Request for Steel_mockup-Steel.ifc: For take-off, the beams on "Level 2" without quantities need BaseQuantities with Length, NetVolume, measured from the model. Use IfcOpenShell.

First a look at what the model holds.

```python
import ifcopenshell
import ifcopenshell.util.element
import ifcopenshell.util.unit

model = ifcopenshell.open("Steel_mockup-Steel.ifc")
print(model.schema)
for unit_type in ("LENGTHUNIT", "AREAUNIT", "VOLUMEUNIT"):
    print(unit_type, ifcopenshell.util.unit.calculate_unit_scale(model, unit_type))
storey = next(s for s in model.by_type("IfcBuildingStorey") if s.Name == "Level 2")
beams = [e for e in ifcopenshell.util.element.get_decomposition(storey) if e.is_a("IfcBeam")]
for e in sorted(beams, key=lambda e: e.id()):
    print(e.id(), e.is_a(), e.Name, list(ifcopenshell.util.element.get_psets(e, qtos_only=True)), sep=" | ")
```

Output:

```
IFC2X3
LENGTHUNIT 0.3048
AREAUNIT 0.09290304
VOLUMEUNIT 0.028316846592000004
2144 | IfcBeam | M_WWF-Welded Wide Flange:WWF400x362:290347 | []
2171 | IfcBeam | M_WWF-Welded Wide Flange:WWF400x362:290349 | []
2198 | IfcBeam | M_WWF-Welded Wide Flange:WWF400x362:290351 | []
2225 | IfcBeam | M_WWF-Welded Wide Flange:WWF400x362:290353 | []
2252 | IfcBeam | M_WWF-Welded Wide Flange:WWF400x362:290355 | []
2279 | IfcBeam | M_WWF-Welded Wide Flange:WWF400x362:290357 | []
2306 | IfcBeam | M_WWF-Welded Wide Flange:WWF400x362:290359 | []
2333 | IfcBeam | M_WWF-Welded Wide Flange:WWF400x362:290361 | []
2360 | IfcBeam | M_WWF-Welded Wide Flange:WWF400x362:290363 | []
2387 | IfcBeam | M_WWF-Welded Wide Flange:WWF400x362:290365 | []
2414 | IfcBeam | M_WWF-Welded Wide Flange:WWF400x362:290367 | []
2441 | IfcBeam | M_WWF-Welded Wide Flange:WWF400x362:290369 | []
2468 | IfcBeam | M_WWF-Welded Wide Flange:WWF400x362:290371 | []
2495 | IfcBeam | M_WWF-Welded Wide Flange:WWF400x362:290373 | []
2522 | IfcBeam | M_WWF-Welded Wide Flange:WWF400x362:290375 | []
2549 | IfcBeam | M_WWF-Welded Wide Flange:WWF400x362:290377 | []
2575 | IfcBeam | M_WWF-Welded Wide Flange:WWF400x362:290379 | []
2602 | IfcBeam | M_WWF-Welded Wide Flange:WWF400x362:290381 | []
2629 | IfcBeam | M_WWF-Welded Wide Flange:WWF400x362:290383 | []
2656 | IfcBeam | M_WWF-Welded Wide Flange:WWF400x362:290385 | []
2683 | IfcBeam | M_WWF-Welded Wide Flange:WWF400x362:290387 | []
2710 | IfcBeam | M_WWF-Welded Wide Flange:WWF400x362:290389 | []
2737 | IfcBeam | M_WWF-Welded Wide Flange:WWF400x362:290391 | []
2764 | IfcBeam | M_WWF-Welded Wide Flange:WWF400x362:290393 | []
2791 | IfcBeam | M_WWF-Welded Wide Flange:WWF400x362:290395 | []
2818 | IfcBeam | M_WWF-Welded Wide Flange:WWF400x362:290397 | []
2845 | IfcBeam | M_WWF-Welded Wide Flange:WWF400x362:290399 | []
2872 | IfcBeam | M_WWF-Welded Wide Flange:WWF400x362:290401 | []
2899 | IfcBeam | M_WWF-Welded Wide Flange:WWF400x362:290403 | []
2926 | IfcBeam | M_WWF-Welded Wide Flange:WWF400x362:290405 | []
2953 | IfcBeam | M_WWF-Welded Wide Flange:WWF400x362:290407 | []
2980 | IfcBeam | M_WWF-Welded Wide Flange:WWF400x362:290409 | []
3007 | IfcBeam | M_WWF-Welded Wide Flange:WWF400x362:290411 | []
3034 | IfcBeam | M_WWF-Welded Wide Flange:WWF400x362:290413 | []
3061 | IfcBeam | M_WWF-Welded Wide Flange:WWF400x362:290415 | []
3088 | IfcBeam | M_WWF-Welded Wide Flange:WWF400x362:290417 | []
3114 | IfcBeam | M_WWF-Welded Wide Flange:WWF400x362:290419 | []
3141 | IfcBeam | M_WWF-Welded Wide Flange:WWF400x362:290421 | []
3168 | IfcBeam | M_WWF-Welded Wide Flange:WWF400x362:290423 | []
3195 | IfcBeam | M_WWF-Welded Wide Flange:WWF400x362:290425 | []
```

```python
import ifcopenshell
import ifcopenshell.api.pset
import ifcopenshell.geom
import ifcopenshell.util.element
import ifcopenshell.util.shape
import ifcopenshell.util.unit

model = ifcopenshell.open("Steel_mockup-Steel.ifc")
unit_scale = ifcopenshell.util.unit.calculate_unit_scale(model)
volume_scale = ifcopenshell.util.unit.calculate_unit_scale(model, "VOLUMEUNIT")
settings = ifcopenshell.geom.settings()

storey = next(s for s in model.by_type("IfcBuildingStorey") if s.Name == "Level 2")
beams = [e for e in ifcopenshell.util.element.get_decomposition(storey) if e.is_a("IfcBeam")]

for e in sorted(beams, key=lambda e: e.id()):
    if ifcopenshell.util.element.get_psets(e, qtos_only=True, should_inherit=False):
        continue
    # Geometry comes back in metres, in the element's own axes.
    shape = ifcopenshell.geom.create_shape(settings, e)
    values = {
        "Length": ifcopenshell.util.shape.get_max_xyz(shape.geometry) / unit_scale,
        "NetVolume": ifcopenshell.util.shape.get_volume(shape.geometry) / volume_scale,
    }
    qto = ifcopenshell.api.pset.add_qto(model, product=e, name="BaseQuantities")
    ifcopenshell.api.pset.edit_qto(model, qto=qto, properties=values)
    print(e.id(), {k: round(v, 3) for k, v in values.items()})

model.write("Steel_mockup-Steel_edited.ifc")
```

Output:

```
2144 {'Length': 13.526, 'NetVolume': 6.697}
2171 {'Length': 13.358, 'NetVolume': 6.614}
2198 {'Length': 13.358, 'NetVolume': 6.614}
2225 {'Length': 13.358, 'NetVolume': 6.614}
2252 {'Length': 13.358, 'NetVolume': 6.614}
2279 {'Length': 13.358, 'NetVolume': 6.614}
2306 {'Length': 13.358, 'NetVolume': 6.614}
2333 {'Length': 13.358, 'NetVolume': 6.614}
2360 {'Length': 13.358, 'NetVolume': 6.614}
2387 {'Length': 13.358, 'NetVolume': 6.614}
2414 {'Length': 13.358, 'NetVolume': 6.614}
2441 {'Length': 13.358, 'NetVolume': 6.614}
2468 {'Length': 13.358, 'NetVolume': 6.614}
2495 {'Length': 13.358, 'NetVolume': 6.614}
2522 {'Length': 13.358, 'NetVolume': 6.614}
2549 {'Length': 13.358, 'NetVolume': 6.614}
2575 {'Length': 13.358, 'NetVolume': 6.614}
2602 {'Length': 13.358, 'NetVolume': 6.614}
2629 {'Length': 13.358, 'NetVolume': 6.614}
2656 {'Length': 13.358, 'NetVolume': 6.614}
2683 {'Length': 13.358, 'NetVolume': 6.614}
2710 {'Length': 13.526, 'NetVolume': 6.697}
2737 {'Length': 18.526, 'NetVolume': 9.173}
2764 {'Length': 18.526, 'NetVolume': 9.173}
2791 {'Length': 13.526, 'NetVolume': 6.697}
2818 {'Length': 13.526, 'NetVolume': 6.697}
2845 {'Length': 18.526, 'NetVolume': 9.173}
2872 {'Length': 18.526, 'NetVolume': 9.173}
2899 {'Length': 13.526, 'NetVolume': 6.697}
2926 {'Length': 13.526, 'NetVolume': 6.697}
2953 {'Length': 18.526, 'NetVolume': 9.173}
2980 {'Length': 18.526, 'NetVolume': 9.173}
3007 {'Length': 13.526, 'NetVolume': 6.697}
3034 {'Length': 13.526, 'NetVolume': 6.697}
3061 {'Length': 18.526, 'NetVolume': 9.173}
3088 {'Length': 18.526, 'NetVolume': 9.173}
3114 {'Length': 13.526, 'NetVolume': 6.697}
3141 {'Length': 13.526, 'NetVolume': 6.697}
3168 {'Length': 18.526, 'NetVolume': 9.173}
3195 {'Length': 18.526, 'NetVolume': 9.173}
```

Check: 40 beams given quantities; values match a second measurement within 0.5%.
